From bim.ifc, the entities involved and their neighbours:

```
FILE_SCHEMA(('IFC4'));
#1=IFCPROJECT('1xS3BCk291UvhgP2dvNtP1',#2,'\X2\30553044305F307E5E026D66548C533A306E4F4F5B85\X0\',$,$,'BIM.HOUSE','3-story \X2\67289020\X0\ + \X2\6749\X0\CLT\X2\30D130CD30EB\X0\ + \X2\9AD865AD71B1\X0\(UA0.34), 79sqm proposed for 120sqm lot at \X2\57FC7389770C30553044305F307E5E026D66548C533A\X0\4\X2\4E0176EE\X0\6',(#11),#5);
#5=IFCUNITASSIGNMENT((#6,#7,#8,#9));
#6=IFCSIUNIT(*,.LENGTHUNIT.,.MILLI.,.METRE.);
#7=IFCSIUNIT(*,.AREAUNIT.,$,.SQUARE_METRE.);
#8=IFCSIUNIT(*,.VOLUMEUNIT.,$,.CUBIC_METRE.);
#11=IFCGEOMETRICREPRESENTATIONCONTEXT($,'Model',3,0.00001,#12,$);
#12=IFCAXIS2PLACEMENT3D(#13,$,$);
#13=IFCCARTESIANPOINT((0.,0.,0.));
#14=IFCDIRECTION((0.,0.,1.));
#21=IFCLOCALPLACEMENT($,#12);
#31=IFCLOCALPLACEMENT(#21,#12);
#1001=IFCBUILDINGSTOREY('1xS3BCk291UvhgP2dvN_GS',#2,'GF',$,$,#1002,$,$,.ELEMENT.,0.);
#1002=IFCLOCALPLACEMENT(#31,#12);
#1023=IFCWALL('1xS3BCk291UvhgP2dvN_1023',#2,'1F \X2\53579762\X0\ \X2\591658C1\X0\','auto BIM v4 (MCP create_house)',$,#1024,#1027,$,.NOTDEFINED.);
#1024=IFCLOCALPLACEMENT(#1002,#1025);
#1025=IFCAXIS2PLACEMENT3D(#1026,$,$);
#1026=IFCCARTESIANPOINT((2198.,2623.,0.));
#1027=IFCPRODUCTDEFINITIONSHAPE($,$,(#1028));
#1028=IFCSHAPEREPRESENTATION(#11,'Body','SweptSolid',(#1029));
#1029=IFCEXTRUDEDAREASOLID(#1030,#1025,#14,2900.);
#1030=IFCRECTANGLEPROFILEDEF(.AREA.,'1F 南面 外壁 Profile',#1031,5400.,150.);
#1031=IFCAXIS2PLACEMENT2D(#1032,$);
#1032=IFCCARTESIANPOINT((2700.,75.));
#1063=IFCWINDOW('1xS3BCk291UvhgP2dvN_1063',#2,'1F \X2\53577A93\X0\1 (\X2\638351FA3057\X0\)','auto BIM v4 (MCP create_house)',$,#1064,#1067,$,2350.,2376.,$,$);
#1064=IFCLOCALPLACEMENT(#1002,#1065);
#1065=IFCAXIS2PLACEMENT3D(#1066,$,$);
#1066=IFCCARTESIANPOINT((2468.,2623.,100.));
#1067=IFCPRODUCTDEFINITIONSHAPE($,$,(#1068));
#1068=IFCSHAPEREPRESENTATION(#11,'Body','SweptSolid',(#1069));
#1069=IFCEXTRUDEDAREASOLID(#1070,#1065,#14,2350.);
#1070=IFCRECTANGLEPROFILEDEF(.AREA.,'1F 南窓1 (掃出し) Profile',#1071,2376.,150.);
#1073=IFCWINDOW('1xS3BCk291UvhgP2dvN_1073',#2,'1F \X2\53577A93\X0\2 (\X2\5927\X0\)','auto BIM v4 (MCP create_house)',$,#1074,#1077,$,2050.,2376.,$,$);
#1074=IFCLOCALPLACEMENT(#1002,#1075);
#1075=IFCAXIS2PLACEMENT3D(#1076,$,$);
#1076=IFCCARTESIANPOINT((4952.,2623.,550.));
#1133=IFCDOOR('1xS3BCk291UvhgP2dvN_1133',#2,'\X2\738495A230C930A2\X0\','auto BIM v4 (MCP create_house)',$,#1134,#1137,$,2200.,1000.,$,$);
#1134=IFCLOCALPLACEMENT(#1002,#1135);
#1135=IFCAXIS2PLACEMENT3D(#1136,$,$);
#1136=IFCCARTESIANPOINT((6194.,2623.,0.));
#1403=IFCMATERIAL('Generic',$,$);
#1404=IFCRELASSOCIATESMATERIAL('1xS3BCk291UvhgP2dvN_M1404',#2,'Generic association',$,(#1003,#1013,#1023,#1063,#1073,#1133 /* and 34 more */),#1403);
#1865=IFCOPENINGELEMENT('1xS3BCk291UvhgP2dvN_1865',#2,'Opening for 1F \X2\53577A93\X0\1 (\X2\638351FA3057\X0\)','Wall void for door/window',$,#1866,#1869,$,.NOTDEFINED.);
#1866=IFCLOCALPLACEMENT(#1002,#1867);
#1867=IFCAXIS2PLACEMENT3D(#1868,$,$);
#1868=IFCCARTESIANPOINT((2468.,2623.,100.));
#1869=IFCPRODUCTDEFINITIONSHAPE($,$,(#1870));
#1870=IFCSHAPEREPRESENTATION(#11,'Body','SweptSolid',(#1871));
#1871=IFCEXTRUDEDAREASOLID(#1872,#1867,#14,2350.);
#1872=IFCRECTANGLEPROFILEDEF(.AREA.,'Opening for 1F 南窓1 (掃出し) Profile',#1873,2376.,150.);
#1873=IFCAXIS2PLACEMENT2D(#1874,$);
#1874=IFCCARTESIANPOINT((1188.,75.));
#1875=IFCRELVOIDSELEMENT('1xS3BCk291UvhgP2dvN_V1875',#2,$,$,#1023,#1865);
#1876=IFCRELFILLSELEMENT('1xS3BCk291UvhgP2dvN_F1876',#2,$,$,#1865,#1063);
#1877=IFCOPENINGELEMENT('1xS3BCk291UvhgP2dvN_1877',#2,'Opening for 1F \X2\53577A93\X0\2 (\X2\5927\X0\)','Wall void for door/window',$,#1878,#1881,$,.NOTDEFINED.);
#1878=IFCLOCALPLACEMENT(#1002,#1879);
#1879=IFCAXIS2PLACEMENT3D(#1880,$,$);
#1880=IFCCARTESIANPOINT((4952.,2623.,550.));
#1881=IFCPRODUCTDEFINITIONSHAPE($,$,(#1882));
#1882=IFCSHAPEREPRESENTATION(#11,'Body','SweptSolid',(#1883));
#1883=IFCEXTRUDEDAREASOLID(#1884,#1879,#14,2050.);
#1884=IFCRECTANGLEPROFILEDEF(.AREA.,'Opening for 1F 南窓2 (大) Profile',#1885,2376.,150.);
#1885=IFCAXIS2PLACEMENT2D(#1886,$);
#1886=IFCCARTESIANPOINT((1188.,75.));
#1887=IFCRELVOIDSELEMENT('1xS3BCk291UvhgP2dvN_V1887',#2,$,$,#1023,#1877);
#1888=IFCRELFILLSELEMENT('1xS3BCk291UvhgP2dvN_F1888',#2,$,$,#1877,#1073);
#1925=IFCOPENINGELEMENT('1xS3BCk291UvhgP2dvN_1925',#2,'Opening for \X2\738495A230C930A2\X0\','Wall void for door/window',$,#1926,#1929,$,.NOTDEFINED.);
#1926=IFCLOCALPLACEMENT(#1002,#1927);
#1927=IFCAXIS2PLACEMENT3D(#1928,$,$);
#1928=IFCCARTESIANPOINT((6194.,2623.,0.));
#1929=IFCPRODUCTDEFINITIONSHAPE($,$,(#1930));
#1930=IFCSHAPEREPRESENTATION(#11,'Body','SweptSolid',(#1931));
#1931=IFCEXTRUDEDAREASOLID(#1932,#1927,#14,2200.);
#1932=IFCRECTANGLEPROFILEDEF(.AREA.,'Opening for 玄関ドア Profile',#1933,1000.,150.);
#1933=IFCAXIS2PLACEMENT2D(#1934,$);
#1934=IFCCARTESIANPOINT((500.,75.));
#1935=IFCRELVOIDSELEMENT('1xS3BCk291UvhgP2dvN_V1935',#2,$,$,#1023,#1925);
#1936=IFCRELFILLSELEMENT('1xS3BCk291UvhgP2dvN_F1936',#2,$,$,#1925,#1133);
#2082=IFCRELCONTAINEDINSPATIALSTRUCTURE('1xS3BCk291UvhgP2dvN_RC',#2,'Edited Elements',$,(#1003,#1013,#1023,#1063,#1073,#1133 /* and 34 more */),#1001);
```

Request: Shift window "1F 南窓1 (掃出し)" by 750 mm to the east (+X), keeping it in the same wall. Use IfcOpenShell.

```python
import ifcopenshell
import ifcopenshell.api.geometry
import ifcopenshell.util.placement
import ifcopenshell.util.unit

model = ifcopenshell.open("bim.ifc")
unit_scale = ifcopenshell.util.unit.calculate_unit_scale(model)

window = model.by_id(1063)
opening = window.FillsVoids[0].RelatingOpeningElement
wall = opening.VoidsElements[0].RelatingBuildingElement

wall_matrix = ifcopenshell.util.placement.get_local_placement(wall.ObjectPlacement)
shift = wall_matrix[:3, 0] * 0.75 / unit_scale
before = ifcopenshell.util.placement.get_local_placement(window.ObjectPlacement)[:3, 3].copy()

# The window is not placed relative to its opening, so move both.
for product in (opening, window):
    matrix = ifcopenshell.util.placement.get_local_placement(product.ObjectPlacement)
    matrix[:3, 3] += shift
    ifcopenshell.api.geometry.edit_object_placement(model, product=product, matrix=matrix, is_si=False)

after = ifcopenshell.util.placement.get_local_placement(window.ObjectPlacement)[:3, 3]
print("window moved by", (after - before).round(3) + 0.0)

model.write("bim-out.ifc")
```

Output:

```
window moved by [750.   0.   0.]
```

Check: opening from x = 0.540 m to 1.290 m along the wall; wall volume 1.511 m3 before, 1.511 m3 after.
